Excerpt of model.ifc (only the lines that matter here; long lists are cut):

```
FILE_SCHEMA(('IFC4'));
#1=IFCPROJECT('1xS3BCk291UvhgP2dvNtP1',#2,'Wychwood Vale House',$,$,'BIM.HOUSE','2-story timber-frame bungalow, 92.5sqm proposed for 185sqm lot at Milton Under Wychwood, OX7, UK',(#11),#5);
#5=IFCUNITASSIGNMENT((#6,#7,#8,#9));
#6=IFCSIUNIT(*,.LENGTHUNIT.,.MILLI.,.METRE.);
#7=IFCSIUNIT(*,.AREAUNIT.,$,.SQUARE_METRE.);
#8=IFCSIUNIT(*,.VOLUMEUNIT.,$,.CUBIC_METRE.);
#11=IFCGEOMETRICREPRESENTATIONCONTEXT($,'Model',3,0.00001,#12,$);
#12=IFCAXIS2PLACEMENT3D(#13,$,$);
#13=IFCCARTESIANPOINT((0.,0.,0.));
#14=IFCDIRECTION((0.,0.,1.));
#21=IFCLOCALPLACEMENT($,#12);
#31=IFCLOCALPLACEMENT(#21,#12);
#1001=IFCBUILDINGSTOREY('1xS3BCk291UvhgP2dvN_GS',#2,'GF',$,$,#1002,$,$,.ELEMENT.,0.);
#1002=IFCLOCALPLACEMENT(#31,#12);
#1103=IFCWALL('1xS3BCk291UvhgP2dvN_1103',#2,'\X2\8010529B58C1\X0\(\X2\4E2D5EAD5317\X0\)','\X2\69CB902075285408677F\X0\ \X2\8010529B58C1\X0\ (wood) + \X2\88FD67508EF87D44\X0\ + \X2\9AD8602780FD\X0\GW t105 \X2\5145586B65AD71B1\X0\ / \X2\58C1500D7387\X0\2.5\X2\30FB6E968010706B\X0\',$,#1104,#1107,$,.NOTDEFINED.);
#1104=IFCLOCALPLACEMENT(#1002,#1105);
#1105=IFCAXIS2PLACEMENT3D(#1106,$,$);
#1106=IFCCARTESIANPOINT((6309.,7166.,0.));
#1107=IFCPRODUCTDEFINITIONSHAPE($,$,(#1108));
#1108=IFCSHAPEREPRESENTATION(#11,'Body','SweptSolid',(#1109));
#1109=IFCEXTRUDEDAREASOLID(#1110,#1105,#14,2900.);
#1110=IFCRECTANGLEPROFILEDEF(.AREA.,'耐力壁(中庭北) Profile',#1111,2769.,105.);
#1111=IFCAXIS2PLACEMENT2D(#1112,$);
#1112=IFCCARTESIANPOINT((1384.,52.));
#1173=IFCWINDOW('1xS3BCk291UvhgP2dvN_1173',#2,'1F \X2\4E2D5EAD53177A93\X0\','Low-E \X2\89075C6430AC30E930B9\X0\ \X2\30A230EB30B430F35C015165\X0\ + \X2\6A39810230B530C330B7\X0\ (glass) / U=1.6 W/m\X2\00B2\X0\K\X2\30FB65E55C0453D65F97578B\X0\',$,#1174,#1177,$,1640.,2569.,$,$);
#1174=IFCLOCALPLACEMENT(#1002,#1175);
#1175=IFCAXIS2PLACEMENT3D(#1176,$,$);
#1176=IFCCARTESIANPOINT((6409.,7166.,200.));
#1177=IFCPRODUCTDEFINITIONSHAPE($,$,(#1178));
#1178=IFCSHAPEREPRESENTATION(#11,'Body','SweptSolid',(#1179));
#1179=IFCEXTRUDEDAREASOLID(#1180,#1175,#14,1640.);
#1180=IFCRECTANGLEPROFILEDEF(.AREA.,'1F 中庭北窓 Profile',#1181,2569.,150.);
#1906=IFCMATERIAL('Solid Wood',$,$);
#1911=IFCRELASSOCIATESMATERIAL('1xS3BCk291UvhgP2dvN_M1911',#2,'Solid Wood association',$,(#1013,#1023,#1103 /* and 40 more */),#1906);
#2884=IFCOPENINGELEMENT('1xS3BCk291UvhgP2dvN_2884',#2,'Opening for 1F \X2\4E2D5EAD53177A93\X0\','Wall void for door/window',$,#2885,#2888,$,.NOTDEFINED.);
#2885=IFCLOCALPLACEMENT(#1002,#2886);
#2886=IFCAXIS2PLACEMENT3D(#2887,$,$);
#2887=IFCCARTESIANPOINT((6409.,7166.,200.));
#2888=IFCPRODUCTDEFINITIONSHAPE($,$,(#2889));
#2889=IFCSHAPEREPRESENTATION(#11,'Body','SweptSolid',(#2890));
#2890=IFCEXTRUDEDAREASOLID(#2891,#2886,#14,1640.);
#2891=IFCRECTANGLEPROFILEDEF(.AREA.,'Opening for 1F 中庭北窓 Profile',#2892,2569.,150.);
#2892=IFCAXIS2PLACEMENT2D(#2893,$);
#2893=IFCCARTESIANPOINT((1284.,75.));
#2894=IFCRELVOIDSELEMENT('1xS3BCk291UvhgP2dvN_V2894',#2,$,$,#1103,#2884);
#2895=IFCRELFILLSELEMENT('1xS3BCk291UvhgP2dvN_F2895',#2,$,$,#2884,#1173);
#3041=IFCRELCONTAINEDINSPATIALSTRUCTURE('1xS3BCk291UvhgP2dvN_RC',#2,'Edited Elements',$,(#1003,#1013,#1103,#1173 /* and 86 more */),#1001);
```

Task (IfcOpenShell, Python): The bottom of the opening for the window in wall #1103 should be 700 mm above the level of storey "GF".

```python
import numpy as np
import ifcopenshell
import ifcopenshell.api.geometry
import ifcopenshell.geom
import ifcopenshell.util.element
import ifcopenshell.util.placement
import ifcopenshell.util.shape
import ifcopenshell.util.unit

model = ifcopenshell.open("model.ifc")
unit_scale = ifcopenshell.util.unit.calculate_unit_scale(model)

window = model.by_guid("1xS3BCk291UvhgP2dvN_1173")
opening = window.FillsVoids[0].RelatingOpeningElement
storey = ifcopenshell.util.element.get_container(window, ifc_class="IfcBuildingStorey")
level = ifcopenshell.util.placement.get_local_placement(storey.ObjectPlacement)[2, 3]

# The opening's origin need not be at the sill, so measure its lowest point.
shape = ifcopenshell.geom.create_shape(ifcopenshell.geom.settings(), opening)
bottom = ifcopenshell.util.shape.get_shape_bottom_elevation(shape, shape.geometry) / unit_scale
dz = level + 0.7 / unit_scale - bottom

shift = np.array([0.0, 0.0, dz])
# The window is not placed relative to its opening, so move both.
for product in (opening, window):
    matrix = ifcopenshell.util.placement.get_local_placement(product.ObjectPlacement)
    matrix[:3, 3] += shift
    ifcopenshell.api.geometry.edit_object_placement(model, product=product, matrix=matrix, is_si=False)

print(f"moved by {dz * unit_scale:+.3f} m")

model.write("model_rev.ifc")
```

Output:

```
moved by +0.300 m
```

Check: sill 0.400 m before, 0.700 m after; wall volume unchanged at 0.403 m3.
